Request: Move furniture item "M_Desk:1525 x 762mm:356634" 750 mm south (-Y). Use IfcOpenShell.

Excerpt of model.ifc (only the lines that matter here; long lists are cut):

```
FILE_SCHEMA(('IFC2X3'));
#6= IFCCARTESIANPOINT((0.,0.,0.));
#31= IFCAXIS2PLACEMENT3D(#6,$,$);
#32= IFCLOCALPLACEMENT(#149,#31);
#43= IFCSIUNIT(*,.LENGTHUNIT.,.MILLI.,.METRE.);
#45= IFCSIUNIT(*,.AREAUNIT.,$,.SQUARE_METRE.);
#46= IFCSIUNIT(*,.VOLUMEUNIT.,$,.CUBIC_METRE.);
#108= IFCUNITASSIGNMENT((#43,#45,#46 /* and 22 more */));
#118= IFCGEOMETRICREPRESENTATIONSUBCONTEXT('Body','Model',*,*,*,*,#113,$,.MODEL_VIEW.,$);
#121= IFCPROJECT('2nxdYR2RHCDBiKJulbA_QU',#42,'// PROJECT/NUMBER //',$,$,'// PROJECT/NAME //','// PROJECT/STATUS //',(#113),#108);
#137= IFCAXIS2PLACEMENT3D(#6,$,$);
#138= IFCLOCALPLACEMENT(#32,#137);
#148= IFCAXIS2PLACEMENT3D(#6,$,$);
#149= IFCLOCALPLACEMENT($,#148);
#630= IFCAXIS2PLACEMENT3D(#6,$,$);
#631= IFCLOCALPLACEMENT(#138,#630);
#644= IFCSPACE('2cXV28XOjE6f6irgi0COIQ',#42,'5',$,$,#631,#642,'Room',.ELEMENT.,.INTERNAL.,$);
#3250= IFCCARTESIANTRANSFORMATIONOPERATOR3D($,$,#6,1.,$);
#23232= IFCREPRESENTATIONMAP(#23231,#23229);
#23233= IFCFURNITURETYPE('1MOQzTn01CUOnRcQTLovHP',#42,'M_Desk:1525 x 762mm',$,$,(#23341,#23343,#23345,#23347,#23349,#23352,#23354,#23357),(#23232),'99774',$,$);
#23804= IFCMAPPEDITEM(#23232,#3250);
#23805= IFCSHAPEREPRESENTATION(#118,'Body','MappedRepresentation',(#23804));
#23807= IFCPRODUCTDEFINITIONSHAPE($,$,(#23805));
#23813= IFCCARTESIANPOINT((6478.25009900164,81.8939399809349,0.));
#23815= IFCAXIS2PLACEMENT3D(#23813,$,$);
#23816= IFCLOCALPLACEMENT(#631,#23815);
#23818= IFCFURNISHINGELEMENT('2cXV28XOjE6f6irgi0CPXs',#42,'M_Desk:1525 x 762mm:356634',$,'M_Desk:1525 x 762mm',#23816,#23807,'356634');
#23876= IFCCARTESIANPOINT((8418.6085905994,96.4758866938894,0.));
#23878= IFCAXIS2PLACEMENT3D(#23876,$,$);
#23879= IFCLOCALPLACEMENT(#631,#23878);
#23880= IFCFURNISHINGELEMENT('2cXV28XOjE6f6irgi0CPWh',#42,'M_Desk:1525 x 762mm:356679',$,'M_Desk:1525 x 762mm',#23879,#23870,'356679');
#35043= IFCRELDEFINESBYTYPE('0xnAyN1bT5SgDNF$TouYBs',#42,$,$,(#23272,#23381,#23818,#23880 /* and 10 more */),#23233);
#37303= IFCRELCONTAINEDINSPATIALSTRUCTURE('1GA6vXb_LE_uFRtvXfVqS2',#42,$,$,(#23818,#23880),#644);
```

```python
import ifcopenshell
import ifcopenshell.api.geometry
import ifcopenshell.util.placement
import ifcopenshell.util.unit

model = ifcopenshell.open("model.ifc")
unit_scale = ifcopenshell.util.unit.calculate_unit_scale(model)

item = model.by_id(23818)
matrix = ifcopenshell.util.placement.get_local_placement(item.ObjectPlacement)
matrix[1, 3] -= 0.75 / unit_scale
ifcopenshell.api.geometry.edit_object_placement(model, product=item, matrix=matrix, is_si=False)

print(ifcopenshell.util.placement.get_local_placement(item.ObjectPlacement).round(3) + 0.0)

model.write("model_edited.ifc")
```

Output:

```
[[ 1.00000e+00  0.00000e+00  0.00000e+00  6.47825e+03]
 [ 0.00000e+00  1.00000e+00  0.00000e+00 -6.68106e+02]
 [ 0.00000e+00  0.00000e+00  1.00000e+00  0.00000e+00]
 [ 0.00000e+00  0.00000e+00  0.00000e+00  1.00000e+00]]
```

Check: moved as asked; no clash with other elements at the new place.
